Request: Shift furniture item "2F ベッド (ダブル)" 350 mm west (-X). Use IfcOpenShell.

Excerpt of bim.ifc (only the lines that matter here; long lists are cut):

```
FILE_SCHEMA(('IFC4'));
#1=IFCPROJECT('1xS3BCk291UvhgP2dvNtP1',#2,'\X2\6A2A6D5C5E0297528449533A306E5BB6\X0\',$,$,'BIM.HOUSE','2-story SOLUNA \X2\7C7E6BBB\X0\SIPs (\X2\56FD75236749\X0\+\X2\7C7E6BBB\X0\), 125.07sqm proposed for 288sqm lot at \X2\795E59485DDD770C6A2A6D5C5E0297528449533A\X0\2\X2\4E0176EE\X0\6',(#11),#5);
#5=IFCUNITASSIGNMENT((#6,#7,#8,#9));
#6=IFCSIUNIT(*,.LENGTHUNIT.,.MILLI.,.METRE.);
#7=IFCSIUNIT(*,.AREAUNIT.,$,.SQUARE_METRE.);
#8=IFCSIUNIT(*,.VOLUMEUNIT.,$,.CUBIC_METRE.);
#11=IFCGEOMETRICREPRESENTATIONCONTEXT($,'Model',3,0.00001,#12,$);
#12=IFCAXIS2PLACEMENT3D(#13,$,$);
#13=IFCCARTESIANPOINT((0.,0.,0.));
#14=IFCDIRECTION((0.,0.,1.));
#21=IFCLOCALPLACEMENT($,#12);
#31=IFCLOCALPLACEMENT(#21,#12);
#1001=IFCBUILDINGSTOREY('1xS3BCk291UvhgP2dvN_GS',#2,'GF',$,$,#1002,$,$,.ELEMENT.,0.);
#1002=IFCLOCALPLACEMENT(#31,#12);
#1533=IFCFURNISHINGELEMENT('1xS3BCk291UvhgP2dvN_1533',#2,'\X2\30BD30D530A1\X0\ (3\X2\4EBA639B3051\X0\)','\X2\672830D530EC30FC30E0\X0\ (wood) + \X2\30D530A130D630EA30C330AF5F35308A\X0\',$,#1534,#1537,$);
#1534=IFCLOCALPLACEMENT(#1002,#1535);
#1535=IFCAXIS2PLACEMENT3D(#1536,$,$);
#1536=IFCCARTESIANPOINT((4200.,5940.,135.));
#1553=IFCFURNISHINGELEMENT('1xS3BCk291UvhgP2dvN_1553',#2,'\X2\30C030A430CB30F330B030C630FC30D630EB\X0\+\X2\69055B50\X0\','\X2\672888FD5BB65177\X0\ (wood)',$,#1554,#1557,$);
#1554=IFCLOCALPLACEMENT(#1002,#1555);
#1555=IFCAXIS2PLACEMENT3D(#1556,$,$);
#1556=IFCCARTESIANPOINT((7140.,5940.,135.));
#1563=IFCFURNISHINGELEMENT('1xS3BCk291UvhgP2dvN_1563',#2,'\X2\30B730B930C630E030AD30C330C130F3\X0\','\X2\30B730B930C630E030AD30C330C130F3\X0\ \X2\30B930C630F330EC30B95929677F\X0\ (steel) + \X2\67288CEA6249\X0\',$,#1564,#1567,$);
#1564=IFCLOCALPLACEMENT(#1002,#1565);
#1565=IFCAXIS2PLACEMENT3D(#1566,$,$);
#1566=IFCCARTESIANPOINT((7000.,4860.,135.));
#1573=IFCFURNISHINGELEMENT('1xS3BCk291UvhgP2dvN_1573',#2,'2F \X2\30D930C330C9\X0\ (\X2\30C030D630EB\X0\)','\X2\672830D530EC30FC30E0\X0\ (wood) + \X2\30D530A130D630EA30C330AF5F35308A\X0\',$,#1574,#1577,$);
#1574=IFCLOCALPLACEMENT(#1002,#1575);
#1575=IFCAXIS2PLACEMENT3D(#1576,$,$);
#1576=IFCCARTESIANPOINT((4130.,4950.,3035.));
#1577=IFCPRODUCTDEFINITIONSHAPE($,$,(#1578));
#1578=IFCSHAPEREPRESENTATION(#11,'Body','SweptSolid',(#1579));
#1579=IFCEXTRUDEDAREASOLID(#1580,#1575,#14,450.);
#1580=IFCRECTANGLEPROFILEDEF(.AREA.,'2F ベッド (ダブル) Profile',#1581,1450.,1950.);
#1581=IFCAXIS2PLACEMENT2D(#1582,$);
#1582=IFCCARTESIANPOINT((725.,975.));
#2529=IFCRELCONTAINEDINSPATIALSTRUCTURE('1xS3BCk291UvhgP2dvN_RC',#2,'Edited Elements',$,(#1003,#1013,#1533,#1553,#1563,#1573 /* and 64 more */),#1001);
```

```python
import ifcopenshell
import ifcopenshell.api.geometry
import ifcopenshell.util.placement
import ifcopenshell.util.unit

model = ifcopenshell.open("bim.ifc")
unit_scale = ifcopenshell.util.unit.calculate_unit_scale(model)

item = model.by_guid("1xS3BCk291UvhgP2dvN_1573")
matrix = ifcopenshell.util.placement.get_local_placement(item.ObjectPlacement)
matrix[0, 3] -= 0.35 / unit_scale
ifcopenshell.api.geometry.edit_object_placement(model, product=item, matrix=matrix, is_si=False)

print(ifcopenshell.util.placement.get_local_placement(item.ObjectPlacement).round(3) + 0.0)

model.write("bim_v2.ifc")
```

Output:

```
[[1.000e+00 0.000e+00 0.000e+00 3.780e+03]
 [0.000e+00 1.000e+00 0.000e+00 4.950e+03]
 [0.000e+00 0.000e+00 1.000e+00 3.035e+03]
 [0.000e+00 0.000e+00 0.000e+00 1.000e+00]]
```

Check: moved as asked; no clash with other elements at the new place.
